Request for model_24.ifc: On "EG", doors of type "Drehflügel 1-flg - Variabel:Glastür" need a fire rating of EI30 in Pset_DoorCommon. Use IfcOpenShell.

First a look at what the model holds.

```python
import ifcopenshell
import ifcopenshell.util.element

model = ifcopenshell.open("model_24.ifc")
print(model.schema)
storey = next(s for s in model.by_type("IfcBuildingStorey") if s.Name == "EG")
doors = [e for e in ifcopenshell.util.element.get_decomposition(storey) if e.is_a("IfcDoor")]
seen = {}
for e in doors:
    element_type = ifcopenshell.util.element.get_type(e)
    key = (element_type.Name if element_type != e and element_type else None, ifcopenshell.util.element.get_pset(e, "Pset_DoorCommon", "FireRating"))
    seen[key] = seen.get(key, 0) + 1
for (name, value), count in sorted(seen.items(), key=str):
    print(count, "x", name, "|", value)
```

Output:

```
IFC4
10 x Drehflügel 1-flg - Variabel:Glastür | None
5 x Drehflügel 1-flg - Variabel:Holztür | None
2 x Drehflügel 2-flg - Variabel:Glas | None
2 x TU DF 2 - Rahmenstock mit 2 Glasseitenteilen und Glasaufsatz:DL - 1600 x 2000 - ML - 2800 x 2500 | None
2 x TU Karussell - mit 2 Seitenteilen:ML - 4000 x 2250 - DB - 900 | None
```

```python
import ifcopenshell
import ifcopenshell.api.pset
import ifcopenshell.util.element

model = ifcopenshell.open("model_24.ifc")

storey = next(s for s in model.by_type("IfcBuildingStorey") if s.Name == "EG")
doors = [e for e in ifcopenshell.util.element.get_decomposition(storey) if e.is_a("IfcDoor")]

count = 0
for e in doors:
    element_type = ifcopenshell.util.element.get_type(e)
    if element_type in (None, e) or element_type.Name != "Drehflügel 1-flg - Variabel:Glastür":
        continue
    # add_pset returns the element's existing set when there is one.
    pset = ifcopenshell.api.pset.add_pset(model, product=e, name="Pset_DoorCommon")
    ifcopenshell.api.pset.edit_pset(model, pset=pset, properties={"FireRating": "EI30"})
    count += 1

print(count, "doors updated")

model.write("model_24_updated.ifc")
```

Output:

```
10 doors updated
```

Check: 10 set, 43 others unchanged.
